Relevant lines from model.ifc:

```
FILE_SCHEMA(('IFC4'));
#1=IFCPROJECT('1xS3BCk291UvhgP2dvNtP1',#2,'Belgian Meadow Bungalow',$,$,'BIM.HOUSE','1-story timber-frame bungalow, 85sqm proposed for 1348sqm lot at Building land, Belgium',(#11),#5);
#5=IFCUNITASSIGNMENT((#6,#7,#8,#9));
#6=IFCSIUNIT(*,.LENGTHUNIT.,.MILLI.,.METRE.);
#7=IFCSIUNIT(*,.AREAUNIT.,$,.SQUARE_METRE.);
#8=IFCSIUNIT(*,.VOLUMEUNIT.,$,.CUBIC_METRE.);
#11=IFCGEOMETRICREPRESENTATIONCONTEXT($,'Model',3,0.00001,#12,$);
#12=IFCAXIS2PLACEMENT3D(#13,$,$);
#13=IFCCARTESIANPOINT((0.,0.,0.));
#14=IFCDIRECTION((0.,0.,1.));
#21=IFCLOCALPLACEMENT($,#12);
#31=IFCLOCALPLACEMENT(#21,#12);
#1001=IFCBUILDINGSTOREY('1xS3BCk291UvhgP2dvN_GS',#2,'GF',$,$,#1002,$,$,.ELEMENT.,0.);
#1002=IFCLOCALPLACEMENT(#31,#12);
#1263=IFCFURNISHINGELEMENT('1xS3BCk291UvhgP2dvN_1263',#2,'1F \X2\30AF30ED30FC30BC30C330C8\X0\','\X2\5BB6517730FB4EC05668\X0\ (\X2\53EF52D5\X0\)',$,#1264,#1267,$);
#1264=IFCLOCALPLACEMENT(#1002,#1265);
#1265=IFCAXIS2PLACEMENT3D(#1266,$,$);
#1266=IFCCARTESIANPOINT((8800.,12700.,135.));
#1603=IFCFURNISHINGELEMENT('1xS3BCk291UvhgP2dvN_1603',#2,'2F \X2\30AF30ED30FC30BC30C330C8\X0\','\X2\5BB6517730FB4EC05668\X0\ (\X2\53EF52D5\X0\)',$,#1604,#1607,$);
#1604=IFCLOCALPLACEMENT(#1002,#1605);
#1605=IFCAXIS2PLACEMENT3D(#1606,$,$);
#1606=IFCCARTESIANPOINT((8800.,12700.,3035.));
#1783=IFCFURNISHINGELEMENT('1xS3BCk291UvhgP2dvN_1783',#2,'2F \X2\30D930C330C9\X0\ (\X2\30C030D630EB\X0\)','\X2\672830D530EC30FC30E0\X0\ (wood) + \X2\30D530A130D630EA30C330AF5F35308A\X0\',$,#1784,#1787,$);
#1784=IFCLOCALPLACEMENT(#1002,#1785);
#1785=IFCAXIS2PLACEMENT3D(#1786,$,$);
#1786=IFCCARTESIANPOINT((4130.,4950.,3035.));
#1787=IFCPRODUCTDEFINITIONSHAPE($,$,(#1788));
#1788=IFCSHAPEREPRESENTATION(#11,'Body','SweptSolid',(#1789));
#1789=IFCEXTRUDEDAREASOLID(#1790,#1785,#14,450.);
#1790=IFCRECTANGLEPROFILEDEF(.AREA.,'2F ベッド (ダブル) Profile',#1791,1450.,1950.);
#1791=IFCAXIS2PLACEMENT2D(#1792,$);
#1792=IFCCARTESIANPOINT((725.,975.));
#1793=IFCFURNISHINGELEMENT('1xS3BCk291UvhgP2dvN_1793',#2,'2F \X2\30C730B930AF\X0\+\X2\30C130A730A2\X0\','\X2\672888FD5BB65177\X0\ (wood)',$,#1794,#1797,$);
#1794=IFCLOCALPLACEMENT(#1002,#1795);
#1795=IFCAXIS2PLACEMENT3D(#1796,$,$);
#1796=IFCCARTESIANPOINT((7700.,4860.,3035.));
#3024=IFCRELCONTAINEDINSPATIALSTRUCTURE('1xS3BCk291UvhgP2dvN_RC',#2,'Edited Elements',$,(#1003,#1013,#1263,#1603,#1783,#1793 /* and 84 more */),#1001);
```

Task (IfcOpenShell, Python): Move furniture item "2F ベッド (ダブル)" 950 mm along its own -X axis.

```python
import ifcopenshell
import ifcopenshell.api.geometry
import ifcopenshell.util.placement

model = ifcopenshell.open("model.ifc")

item = model.by_guid("1xS3BCk291UvhgP2dvN_1783")
matrix = ifcopenshell.util.placement.get_local_placement(item.ObjectPlacement)
matrix[:3, 3] -= matrix[:3, 0] * 950.0
ifcopenshell.api.geometry.edit_object_placement(model, product=item, matrix=matrix, is_si=False)

print(ifcopenshell.util.placement.get_local_placement(item.ObjectPlacement).round(3) + 0.0)

model.write("model_v2.ifc")
```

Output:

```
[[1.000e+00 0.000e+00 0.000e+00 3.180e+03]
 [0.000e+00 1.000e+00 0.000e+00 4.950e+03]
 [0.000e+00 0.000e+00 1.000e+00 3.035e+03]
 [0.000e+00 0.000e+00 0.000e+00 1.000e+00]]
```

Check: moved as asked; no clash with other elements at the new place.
